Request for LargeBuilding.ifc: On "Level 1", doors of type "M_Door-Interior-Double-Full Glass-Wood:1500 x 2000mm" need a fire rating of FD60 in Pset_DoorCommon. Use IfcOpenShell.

First a look at what the model holds.

```python
import ifcopenshell
import ifcopenshell.util.element

model = ifcopenshell.open("LargeBuilding.ifc")
print(model.schema)
storey = next(s for s in model.by_type("IfcBuildingStorey") if s.Name == "Level 1")
doors = [e for e in ifcopenshell.util.element.get_decomposition(storey) if e.is_a("IfcDoor")]
seen = {}
for e in doors:
    element_type = ifcopenshell.util.element.get_type(e)
    key = (element_type.Name if element_type != e and element_type else None, ifcopenshell.util.element.get_pset(e, "Pset_DoorCommon", "FireRating"))
    seen[key] = seen.get(key, 0) + 1
for (name, value), count in sorted(seen.items(), key=str):
    print(count, "x", name, "|", value)
```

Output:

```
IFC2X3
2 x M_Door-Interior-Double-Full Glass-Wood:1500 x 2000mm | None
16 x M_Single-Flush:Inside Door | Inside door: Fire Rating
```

```python
import ifcopenshell
import ifcopenshell.api.pset
import ifcopenshell.util.element

model = ifcopenshell.open("LargeBuilding.ifc")

storey = next(s for s in model.by_type("IfcBuildingStorey") if s.Name == "Level 1")
doors = [e for e in ifcopenshell.util.element.get_decomposition(storey) if e.is_a("IfcDoor")]

count = 0
for e in doors:
    element_type = ifcopenshell.util.element.get_type(e)
    if element_type in (None, e) or element_type.Name != "M_Door-Interior-Double-Full Glass-Wood:1500 x 2000mm":
        continue
    # add_pset returns the element's existing set when there is one.
    pset = ifcopenshell.api.pset.add_pset(model, product=e, name="Pset_DoorCommon")
    ifcopenshell.api.pset.edit_pset(model, pset=pset, properties={"FireRating": "FD60"})
    count += 1

print(count, "doors updated")

model.write("LargeBuilding-out.ifc")
```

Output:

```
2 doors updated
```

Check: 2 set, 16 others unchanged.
